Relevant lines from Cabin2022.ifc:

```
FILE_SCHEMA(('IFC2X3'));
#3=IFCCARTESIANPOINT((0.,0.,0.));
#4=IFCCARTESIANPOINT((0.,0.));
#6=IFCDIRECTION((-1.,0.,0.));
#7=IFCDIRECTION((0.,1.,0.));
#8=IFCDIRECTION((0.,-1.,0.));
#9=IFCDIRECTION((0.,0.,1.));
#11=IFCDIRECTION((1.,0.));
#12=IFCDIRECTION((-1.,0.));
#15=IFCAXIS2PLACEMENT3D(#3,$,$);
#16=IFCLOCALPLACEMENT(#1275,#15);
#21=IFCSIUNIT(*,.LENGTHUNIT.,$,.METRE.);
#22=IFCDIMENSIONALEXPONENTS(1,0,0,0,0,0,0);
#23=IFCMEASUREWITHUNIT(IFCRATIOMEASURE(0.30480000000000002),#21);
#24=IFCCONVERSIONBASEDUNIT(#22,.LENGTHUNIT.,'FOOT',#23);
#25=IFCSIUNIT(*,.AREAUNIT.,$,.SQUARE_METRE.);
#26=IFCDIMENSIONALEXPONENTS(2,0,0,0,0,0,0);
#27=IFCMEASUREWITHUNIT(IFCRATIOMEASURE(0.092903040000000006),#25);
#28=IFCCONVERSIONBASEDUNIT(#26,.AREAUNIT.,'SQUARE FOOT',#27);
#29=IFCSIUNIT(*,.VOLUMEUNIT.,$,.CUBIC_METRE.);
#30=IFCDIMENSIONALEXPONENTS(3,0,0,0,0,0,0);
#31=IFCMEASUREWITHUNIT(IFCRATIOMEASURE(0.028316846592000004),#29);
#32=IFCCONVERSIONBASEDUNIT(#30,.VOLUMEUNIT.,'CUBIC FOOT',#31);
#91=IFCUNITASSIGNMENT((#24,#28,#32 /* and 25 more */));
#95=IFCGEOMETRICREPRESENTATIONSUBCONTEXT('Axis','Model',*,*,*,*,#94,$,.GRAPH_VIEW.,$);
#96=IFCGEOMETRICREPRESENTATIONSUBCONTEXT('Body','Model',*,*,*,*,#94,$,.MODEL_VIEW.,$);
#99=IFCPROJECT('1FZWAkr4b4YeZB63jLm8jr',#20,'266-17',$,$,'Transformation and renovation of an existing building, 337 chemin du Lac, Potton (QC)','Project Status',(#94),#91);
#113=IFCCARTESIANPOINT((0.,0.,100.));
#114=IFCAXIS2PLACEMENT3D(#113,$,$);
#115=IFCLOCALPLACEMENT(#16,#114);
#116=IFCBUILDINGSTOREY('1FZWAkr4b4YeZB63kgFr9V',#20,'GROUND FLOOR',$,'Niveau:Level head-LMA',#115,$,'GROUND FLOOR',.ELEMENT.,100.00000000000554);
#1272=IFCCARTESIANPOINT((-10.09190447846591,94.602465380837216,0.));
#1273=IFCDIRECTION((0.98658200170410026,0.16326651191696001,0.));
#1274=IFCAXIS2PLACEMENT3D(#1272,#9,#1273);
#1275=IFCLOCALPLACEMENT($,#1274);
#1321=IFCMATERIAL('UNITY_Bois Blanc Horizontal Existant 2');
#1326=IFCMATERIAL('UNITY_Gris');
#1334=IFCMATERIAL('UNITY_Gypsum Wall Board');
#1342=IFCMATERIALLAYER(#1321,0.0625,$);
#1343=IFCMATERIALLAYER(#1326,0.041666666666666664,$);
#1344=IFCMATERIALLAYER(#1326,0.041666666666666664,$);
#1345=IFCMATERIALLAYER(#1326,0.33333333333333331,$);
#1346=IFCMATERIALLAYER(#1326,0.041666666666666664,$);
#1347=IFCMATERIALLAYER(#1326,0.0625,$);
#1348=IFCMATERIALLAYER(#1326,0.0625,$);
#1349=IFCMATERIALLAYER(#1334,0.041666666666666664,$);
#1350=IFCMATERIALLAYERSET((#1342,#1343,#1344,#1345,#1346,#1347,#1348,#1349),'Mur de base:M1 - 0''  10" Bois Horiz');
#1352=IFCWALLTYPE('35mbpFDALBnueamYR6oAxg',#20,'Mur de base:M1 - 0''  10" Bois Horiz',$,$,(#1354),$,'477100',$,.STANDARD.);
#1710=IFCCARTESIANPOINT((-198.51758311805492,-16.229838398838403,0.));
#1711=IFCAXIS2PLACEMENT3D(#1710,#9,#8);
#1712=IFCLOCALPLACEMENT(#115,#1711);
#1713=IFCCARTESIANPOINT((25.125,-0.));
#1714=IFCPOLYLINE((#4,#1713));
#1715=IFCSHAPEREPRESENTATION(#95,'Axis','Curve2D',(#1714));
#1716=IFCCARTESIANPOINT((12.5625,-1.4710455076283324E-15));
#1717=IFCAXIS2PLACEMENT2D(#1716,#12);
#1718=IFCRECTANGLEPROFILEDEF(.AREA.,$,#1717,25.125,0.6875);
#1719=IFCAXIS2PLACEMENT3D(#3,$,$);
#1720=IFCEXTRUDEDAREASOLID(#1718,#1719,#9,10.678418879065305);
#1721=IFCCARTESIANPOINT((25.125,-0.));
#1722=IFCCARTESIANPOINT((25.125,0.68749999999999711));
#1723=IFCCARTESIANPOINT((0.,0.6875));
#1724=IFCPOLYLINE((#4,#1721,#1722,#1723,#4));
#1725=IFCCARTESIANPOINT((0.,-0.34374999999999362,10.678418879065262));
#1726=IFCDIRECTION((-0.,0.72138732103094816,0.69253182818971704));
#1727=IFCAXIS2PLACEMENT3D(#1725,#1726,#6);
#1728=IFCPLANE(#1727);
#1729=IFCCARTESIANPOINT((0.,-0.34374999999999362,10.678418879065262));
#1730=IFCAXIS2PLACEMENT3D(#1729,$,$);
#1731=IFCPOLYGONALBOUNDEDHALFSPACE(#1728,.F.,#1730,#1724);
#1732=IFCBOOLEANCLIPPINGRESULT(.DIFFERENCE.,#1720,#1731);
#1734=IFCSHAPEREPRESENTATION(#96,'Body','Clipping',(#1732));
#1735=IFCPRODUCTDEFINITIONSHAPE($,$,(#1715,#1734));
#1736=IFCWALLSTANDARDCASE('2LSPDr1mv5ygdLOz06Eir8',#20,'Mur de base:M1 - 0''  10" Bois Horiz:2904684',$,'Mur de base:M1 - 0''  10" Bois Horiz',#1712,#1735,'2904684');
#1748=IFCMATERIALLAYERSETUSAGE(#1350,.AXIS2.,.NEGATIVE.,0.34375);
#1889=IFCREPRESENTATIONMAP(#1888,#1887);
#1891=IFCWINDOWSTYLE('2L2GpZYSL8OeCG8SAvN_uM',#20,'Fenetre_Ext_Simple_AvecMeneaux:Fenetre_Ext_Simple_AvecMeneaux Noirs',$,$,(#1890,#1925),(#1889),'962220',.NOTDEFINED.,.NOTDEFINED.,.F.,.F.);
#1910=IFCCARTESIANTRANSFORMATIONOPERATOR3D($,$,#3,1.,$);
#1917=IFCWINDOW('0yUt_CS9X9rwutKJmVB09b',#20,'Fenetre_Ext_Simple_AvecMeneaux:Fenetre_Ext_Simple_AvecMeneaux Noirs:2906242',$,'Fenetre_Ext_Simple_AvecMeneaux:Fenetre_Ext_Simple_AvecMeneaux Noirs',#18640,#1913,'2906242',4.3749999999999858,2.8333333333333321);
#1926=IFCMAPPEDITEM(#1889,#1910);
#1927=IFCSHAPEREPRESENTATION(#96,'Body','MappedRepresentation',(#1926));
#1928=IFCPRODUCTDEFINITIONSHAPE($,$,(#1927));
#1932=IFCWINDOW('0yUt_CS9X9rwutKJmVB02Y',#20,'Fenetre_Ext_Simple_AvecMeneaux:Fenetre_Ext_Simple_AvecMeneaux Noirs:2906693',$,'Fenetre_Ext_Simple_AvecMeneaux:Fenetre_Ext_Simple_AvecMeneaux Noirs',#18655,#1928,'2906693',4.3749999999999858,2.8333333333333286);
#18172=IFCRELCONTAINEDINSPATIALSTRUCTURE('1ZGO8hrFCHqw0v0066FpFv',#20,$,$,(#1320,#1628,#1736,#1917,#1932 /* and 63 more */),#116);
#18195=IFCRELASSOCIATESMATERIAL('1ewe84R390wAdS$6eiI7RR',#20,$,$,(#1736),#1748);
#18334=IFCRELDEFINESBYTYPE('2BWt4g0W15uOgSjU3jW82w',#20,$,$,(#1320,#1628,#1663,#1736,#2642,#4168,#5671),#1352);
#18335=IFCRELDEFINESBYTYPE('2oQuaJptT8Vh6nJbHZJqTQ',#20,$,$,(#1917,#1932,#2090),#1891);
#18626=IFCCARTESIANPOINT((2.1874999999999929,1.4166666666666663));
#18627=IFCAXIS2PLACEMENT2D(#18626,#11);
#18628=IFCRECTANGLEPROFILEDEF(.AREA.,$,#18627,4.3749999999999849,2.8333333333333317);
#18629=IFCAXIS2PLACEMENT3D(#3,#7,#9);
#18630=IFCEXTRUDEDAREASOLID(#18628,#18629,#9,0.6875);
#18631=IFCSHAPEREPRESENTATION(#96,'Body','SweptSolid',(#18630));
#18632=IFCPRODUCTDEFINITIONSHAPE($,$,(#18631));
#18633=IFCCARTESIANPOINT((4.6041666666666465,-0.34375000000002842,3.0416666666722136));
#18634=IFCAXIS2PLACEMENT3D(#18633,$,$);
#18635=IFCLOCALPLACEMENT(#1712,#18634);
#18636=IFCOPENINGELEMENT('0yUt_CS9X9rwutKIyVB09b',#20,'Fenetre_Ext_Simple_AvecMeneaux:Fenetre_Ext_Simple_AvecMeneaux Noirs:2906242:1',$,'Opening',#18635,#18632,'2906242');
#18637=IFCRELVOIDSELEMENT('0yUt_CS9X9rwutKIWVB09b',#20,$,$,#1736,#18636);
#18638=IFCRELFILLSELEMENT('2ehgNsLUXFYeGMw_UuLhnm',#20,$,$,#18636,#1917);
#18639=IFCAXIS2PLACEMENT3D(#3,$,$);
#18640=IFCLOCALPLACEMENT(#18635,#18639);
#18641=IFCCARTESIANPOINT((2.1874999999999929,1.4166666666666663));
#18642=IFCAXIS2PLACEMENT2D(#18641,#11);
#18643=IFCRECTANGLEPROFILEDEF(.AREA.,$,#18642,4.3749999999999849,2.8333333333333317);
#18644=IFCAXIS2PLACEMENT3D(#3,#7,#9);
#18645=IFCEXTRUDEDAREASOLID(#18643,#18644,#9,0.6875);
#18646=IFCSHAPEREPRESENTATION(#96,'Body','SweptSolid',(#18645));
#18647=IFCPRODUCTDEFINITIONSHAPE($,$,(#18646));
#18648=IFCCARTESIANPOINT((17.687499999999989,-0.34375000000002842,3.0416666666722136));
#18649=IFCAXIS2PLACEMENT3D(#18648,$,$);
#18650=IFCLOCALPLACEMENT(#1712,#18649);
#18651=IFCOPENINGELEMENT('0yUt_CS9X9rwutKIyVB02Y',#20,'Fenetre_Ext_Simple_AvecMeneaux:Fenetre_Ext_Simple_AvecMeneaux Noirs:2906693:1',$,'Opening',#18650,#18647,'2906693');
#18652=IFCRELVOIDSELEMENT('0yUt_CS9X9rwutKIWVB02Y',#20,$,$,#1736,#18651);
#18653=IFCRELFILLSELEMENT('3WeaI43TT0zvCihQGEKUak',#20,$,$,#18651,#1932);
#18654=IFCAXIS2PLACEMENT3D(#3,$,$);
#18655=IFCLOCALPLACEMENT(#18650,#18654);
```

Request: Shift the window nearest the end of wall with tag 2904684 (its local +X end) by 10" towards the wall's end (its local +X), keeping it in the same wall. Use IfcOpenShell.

```python
import ifcopenshell
import ifcopenshell.api.geometry
import ifcopenshell.util.placement
import ifcopenshell.util.unit

model = ifcopenshell.open("Cabin2022.ifc")
unit_scale = ifcopenshell.util.unit.calculate_unit_scale(model)

window = model.by_id(1932)
opening = window.FillsVoids[0].RelatingOpeningElement
wall = opening.VoidsElements[0].RelatingBuildingElement

wall_matrix = ifcopenshell.util.placement.get_local_placement(wall.ObjectPlacement)
shift = wall_matrix[:3, 0] * 10 * 0.0254 / unit_scale
before = ifcopenshell.util.placement.get_local_placement(window.ObjectPlacement)[:3, 3].copy()

# The window is placed relative to its opening, so it follows when the opening moves.
matrix = ifcopenshell.util.placement.get_local_placement(opening.ObjectPlacement)
matrix[:3, 3] += shift
ifcopenshell.api.geometry.edit_object_placement(
    model, product=opening, matrix=matrix, is_si=False, should_transform_children=True
)

after = ifcopenshell.util.placement.get_local_placement(window.ObjectPlacement)[:3, 3]
print("window moved by", (after - before).round(3) + 0.0)

model.write("Cabin2022_v2.ifc")
```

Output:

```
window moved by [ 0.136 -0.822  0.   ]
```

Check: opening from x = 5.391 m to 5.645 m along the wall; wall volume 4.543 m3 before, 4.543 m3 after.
